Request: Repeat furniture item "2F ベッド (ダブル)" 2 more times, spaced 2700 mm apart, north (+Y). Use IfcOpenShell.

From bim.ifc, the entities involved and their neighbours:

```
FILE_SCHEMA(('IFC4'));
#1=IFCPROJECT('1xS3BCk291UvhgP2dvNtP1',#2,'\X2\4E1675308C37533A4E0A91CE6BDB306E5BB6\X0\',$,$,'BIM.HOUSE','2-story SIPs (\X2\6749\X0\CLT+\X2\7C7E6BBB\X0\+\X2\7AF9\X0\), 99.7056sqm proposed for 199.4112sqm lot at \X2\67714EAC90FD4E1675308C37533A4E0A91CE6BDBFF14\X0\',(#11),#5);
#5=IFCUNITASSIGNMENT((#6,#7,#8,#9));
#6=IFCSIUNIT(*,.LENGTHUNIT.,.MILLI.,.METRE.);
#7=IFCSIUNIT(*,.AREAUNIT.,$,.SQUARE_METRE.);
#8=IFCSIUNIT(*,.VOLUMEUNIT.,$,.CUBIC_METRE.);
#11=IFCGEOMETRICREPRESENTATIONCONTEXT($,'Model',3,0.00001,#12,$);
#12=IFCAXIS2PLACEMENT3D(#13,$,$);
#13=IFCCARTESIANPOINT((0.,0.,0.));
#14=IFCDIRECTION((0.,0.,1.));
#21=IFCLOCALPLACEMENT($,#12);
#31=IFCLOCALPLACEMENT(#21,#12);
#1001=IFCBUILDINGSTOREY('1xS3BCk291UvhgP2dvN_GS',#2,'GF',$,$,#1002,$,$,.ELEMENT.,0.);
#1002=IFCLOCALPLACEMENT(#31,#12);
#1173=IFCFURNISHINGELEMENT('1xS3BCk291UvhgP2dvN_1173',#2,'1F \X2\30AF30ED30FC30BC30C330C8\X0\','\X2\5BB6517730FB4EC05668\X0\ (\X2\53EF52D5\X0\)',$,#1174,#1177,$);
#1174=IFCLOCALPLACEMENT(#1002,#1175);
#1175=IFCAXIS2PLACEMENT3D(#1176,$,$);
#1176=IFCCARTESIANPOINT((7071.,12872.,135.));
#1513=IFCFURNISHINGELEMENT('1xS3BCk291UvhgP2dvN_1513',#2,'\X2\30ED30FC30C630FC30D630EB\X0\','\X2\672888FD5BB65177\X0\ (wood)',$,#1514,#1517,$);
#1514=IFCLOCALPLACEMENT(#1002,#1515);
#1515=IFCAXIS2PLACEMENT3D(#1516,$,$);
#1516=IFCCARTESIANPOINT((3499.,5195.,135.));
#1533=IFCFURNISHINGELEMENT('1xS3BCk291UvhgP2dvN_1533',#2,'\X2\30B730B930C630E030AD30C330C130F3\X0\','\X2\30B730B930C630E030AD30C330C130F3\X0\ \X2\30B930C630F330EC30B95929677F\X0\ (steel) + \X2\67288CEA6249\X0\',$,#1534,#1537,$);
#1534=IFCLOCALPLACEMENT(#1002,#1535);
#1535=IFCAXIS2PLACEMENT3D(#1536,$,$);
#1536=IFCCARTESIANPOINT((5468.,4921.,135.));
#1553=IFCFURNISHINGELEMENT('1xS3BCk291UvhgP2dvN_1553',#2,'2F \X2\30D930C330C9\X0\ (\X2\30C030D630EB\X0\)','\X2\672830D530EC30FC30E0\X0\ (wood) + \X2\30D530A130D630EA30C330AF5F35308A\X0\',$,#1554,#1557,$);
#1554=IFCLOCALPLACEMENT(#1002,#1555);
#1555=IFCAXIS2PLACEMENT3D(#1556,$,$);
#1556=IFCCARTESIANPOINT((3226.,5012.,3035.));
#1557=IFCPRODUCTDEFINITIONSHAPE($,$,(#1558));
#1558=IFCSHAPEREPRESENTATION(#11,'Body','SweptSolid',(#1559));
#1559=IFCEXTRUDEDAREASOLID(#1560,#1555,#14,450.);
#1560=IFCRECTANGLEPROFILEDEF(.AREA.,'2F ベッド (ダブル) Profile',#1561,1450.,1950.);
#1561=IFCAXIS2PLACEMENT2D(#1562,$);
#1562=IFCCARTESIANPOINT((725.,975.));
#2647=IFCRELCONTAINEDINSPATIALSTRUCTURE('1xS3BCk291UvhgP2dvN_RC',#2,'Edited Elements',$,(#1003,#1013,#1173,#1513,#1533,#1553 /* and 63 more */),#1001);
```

```python
import numpy as np
import ifcopenshell
import ifcopenshell.api.geometry
import ifcopenshell.api.root
import ifcopenshell.util.element
import ifcopenshell.util.placement

model = ifcopenshell.open("bim.ifc")


def reuse_history(source, copy):
    """copy_class also copies each property set's owner history, people and application; keep the originals."""
    for rel in copy.IsDefinedBy:
        if rel.is_a("IfcRelDefinesByProperties") and (history := rel.RelatingPropertyDefinition.OwnerHistory):
            rel.RelatingPropertyDefinition.OwnerHistory = source.OwnerHistory
            ifcopenshell.util.element.remove_deep2(model, history)


source = model.by_guid("1xS3BCk291UvhgP2dvN_1553")
base = ifcopenshell.util.placement.get_local_placement(source.ObjectPlacement)
step = np.array([0.0, 1.0, 0.0]) * 2700.0

for i in range(1, 3):
    copy = ifcopenshell.api.root.copy_class(model, product=source)
    copy.Representation = ifcopenshell.util.element.copy_deep(
        model, source.Representation, exclude=["IfcGeometricRepresentationContext", "IfcRepresentationMap"]
    )
    reuse_history(source, copy)
    matrix = base.copy()
    matrix[:3, 3] += i * step
    print("added at", matrix[:3, 3].round(3) + 0.0)
    ifcopenshell.api.geometry.edit_object_placement(model, product=copy, matrix=matrix, is_si=False)

model.write("bim_v2.ifc")
```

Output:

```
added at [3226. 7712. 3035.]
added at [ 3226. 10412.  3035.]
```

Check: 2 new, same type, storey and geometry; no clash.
